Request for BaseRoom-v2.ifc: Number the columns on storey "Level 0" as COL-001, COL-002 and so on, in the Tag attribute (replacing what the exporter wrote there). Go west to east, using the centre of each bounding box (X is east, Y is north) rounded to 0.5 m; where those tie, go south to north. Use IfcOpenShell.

First a look at what the model holds.

```python
import ifcopenshell
import ifcopenshell.util.element
import ifcopenshell.util.placement

model = ifcopenshell.open("BaseRoom-v2.ifc")
print(model.schema)
storey = next(s for s in model.by_type("IfcBuildingStorey") if s.Name == "Level 0")
columns = [e for e in ifcopenshell.util.element.get_decomposition(storey) if e.is_a("IfcColumn")]
for e in sorted(columns, key=lambda e: e.id()):
    origin = ifcopenshell.util.placement.get_local_placement(e.ObjectPlacement)[:3, 3]
    print(e.id(), e.Tag, e.Name, origin.round(2) + 0.0, sep=" | ")
```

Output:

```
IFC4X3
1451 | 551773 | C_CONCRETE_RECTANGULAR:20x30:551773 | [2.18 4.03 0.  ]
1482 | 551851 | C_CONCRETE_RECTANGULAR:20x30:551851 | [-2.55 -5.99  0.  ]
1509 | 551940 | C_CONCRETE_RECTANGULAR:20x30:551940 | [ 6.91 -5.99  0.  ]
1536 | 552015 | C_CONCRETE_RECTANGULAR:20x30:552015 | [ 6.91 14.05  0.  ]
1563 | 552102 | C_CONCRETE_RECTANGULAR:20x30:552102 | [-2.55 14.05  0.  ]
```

```python
import ifcopenshell
import ifcopenshell.geom
import ifcopenshell.util.element
import ifcopenshell.util.shape

model = ifcopenshell.open("BaseRoom-v2.ifc")
settings = ifcopenshell.geom.settings()
settings.set("use-world-coords", True)


def centre(element):
    shape = ifcopenshell.geom.create_shape(settings, element)
    return ifcopenshell.util.shape.get_bbox_centroid(shape.geometry)


storey = next(s for s in model.by_type("IfcBuildingStorey") if s.Name == "Level 0")
columns = [e for e in ifcopenshell.util.element.get_decomposition(storey) if e.is_a("IfcColumn")]

# Insertion points can sit at a corner or the storey origin, so sort by the geometry (in metres).
centres = {e: centre(e) for e in columns}
columns.sort(key=lambda e: (round(centres[e][0] / 0.5), centres[e][1]))

for i, e in enumerate(columns, start=1):
    number = f"COL-0{i:02d}"
    e.Tag = number
    print(e.id(), number)

model.write("BaseRoom-v2_v2.ifc")
```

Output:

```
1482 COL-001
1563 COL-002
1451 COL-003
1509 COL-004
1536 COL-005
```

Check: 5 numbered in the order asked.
